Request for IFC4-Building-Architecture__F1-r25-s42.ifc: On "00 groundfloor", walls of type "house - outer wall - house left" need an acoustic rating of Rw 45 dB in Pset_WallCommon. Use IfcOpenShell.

First a look at what the model holds.

```python
import ifcopenshell
import ifcopenshell.util.element

model = ifcopenshell.open("IFC4-Building-Architecture__F1-r25-s42.ifc")
print(model.schema)
storey = next(s for s in model.by_type("IfcBuildingStorey") if s.Name == "00 groundfloor")
walls = [e for e in ifcopenshell.util.element.get_decomposition(storey) if e.is_a("IfcWall")]
seen = {}
for e in walls:
    element_type = ifcopenshell.util.element.get_type(e)
    key = (element_type.Name if element_type != e and element_type else None, ifcopenshell.util.element.get_pset(e, "Pset_WallCommon", "AcousticRating"))
    seen[key] = seen.get(key, 0) + 1
for (name, value), count in sorted(seen.items(), key=str):
    print(count, "x", name, "|", value)
```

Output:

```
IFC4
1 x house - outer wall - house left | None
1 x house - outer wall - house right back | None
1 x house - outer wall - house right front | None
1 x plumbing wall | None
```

```python
import ifcopenshell
import ifcopenshell.api.pset
import ifcopenshell.util.element

model = ifcopenshell.open("IFC4-Building-Architecture__F1-r25-s42.ifc")

storey = next(s for s in model.by_type("IfcBuildingStorey") if s.Name == "00 groundfloor")
walls = [e for e in ifcopenshell.util.element.get_decomposition(storey) if e.is_a("IfcWall")]

count = 0
for e in walls:
    element_type = ifcopenshell.util.element.get_type(e)
    if element_type in (None, e) or element_type.Name != "house - outer wall - house left":
        continue
    # add_pset returns the element's existing set when there is one.
    pset = ifcopenshell.api.pset.add_pset(model, product=e, name="Pset_WallCommon")
    ifcopenshell.api.pset.edit_pset(model, pset=pset, properties={"AcousticRating": "Rw 45 dB"})
    count += 1

print(count, "walls updated")

model.write("IFC4-Building-Architecture__F1-r25-s42_rev.ifc")
```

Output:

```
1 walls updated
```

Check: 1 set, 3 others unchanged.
